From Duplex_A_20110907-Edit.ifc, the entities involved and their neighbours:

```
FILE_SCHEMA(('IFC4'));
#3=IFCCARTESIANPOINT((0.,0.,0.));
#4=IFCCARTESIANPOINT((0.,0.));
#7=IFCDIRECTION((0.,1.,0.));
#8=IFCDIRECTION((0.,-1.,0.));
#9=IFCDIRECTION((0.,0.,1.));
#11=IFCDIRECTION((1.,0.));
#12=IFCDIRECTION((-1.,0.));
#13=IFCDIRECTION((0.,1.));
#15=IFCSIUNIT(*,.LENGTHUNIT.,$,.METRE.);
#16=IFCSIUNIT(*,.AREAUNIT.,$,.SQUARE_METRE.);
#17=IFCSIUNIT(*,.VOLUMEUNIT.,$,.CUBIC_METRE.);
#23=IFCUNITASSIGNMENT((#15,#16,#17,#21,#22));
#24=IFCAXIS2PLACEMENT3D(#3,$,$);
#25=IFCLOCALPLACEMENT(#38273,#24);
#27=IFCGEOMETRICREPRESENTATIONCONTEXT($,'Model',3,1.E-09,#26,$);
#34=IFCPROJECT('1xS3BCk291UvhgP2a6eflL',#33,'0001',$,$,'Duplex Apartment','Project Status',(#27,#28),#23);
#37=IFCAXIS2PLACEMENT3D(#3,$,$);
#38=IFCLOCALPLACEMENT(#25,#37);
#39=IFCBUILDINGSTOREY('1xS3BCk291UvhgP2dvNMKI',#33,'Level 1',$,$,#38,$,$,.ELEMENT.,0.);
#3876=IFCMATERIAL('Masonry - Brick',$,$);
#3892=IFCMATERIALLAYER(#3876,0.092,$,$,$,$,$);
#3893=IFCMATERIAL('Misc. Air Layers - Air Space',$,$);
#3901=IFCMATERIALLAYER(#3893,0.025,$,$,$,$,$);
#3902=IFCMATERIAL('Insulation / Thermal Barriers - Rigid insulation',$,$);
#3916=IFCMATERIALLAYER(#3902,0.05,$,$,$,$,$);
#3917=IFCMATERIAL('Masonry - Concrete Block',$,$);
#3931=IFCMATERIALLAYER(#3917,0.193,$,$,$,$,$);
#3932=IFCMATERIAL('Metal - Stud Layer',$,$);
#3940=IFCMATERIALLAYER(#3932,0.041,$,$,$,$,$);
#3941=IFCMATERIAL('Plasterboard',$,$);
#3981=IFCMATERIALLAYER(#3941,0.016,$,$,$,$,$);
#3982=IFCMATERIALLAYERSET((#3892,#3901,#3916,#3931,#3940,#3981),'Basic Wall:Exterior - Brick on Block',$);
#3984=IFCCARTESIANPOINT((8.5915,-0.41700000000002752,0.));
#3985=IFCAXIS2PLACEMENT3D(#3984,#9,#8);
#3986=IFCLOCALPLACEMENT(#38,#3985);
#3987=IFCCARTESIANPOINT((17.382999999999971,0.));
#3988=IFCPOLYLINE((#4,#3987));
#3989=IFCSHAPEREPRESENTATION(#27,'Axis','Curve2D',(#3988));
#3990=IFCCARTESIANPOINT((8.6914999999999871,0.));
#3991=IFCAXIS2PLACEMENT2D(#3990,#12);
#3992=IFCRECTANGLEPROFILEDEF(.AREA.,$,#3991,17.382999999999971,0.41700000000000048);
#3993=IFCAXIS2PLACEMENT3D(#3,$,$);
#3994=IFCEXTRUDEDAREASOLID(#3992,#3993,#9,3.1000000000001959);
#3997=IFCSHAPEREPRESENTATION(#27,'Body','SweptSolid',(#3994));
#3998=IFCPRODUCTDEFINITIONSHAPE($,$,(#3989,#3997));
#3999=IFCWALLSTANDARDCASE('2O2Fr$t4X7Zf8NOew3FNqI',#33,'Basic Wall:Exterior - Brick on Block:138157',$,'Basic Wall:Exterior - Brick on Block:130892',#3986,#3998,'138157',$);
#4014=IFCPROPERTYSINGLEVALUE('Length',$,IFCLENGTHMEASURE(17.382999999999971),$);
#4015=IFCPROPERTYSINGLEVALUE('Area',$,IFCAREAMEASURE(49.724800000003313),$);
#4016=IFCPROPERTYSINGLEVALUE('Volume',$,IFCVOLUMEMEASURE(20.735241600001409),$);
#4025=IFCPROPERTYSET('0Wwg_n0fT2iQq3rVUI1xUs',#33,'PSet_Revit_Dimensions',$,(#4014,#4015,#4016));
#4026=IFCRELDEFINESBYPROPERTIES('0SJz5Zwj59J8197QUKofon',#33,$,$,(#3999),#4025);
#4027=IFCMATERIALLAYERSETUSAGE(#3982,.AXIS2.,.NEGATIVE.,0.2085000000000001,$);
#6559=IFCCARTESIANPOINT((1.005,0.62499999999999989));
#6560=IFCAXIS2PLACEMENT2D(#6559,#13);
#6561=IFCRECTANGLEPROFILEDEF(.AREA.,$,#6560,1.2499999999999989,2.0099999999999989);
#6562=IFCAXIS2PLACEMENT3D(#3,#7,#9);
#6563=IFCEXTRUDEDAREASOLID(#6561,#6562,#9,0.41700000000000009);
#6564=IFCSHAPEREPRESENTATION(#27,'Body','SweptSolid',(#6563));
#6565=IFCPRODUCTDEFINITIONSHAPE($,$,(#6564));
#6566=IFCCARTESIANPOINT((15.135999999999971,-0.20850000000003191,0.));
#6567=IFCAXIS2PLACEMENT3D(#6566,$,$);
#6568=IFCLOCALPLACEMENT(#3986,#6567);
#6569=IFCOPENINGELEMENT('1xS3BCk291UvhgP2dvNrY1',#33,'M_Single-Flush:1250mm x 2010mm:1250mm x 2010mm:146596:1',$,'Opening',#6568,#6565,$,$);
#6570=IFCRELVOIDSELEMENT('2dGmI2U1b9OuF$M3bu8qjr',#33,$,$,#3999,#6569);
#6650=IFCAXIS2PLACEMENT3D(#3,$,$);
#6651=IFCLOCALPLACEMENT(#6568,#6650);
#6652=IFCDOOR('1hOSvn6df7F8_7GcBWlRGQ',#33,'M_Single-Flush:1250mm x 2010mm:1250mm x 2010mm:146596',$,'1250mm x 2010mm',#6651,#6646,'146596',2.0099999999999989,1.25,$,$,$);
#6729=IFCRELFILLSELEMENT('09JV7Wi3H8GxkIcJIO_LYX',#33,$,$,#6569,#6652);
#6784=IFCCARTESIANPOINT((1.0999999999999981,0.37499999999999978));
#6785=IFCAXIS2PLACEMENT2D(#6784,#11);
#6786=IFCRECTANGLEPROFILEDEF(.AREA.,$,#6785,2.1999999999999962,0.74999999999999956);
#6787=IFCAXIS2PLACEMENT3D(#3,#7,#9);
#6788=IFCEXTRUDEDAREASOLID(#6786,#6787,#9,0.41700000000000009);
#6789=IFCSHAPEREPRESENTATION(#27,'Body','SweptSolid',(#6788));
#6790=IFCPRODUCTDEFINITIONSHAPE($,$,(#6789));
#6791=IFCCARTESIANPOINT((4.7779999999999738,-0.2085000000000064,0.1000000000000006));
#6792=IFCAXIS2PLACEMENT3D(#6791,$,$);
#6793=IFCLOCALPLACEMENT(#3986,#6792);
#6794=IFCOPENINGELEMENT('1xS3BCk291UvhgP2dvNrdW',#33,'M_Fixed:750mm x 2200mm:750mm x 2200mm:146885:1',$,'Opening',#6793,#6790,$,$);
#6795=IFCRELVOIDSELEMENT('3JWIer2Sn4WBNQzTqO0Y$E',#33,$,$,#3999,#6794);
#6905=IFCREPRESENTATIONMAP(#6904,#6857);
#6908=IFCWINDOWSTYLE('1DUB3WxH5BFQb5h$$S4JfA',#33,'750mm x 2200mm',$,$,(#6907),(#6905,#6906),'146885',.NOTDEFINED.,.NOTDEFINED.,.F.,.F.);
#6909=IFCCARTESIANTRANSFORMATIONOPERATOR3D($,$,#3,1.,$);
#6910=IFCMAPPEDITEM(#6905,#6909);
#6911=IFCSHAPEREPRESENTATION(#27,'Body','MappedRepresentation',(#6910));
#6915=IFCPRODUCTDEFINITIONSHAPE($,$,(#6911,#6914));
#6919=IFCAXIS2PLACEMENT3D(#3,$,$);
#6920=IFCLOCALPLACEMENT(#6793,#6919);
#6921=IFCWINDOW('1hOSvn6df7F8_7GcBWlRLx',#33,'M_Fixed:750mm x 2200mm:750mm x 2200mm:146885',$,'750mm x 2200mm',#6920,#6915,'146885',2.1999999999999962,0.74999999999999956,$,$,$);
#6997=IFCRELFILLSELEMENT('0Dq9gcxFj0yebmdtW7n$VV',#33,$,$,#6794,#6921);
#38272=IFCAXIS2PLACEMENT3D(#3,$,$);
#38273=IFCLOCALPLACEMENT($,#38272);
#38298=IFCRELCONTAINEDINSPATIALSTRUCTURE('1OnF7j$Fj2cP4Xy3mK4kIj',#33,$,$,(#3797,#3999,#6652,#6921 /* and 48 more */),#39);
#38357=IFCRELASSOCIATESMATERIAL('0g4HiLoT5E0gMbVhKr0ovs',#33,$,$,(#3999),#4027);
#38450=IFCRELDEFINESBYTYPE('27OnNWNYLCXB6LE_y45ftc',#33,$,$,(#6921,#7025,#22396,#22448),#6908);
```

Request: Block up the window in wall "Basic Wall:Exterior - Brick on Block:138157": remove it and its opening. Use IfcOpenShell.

```python
import ifcopenshell
import ifcopenshell.api.feature
import ifcopenshell.api.pset
import ifcopenshell.api.root
import ifcopenshell.geom
import ifcopenshell.util.element
import ifcopenshell.util.shape
import ifcopenshell.util.unit

model = ifcopenshell.open("Duplex_A_20110907-Edit.ifc")
area_scale = ifcopenshell.util.unit.calculate_unit_scale(model, "AREAUNIT")
volume_scale = ifcopenshell.util.unit.calculate_unit_scale(model, "VOLUMEUNIT")
settings = ifcopenshell.geom.settings()


def volume(element):
    """Net volume in cubic metres, openings subtracted."""
    shape = ifcopenshell.geom.create_shape(settings, element)
    return ifcopenshell.util.shape.get_volume(shape.geometry)


window = model.by_guid("1hOSvn6df7F8_7GcBWlRLx")
opening = window.FillsVoids[0].RelatingOpeningElement
wall = opening.VoidsElements[0].RelatingBuildingElement
before = volume(wall)

ifcopenshell.api.root.remove_product(model, product=window)
ifcopenshell.api.feature.remove_feature(model, feature=opening)

after = volume(wall)
thickness = 0.417  # wall thickness in metres

# Update the wall's stored quantities.
pset = model.by_id(ifcopenshell.util.element.get_pset(wall, "PSet_Revit_Dimensions", should_inherit=False)["id"])
ifcopenshell.api.pset.edit_pset(model, pset=pset, properties={
    "Area": model.create_entity("IfcAreaMeasure", after / thickness / area_scale),
    "Volume": model.create_entity("IfcVolumeMeasure", after / volume_scale),
})

print(f"wall volume {before:.3f} -> {after:.3f} m3")

model.write("Duplex_A_20110907-Edit_edited.ifc")
```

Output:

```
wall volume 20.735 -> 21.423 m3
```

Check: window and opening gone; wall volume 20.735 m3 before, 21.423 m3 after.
